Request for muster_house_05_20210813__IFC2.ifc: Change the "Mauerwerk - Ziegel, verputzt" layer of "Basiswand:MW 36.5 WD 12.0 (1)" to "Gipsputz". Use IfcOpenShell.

First a look at what the model holds.

```python
import ifcopenshell
import ifcopenshell.util.element

model = ifcopenshell.open("muster_house_05_20210813__IFC2.ifc")
print(model.schema)
for layer_set in model.by_type("IfcMaterialLayerSet"):
    if layer_set.LayerSetName == "Basiswand:MW 36.5 WD 12.0 (1)":
        for layer in layer_set.MaterialLayers:
            print(layer.id(), layer.Material and layer.Material.Name, layer.LayerThickness, sep=" | ")
        print(len(ifcopenshell.util.element.get_elements_by_material(model, layer_set)), "elements and types use it")
print(sorted(m.Name for m in model.by_type("IfcMaterial") if m.Name)[:60])
```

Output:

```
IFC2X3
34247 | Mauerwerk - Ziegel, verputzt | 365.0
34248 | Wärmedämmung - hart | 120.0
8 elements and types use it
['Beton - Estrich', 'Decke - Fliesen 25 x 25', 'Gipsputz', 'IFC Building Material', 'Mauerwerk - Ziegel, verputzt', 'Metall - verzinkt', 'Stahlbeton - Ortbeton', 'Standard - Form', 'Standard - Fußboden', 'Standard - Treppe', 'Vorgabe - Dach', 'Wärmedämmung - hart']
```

```python
import ifcopenshell
import ifcopenshell.api.material

model = ifcopenshell.open("muster_house_05_20210813__IFC2.ifc")

layer_set = next(s for s in model.by_type("IfcMaterialLayerSet") if s.LayerSetName == "Basiswand:MW 36.5 WD 12.0 (1)")
layer = next(l for l in layer_set.MaterialLayers if l.Material and l.Material.Name == "Mauerwerk - Ziegel, verputzt")
material = next(m for m in model.by_type("IfcMaterial") if m.Name == "Gipsputz")

# Point this one layer at the other material; renaming the old one would change it everywhere.
ifcopenshell.api.material.edit_layer(model, layer=layer, attributes={}, material=material)

print([l.Material.Name if l.Material else None for l in layer_set.MaterialLayers])

model.write("muster_house_05_20210813__IFC2_rev.ifc")
```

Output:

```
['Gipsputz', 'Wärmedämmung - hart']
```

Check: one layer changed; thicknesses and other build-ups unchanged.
